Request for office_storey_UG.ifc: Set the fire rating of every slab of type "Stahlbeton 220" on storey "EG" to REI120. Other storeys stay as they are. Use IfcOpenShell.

First a look at what the model holds.

```python
import ifcopenshell
import ifcopenshell.util.element

model = ifcopenshell.open("office_storey_UG.ifc")
print(model.schema)
storey = next(s for s in model.by_type("IfcBuildingStorey") if s.Name == "EG")
slabs = [e for e in ifcopenshell.util.element.get_decomposition(storey) if e.is_a("IfcSlab")]
seen = {}
for e in slabs:
    element_type = ifcopenshell.util.element.get_type(e)
    key = (element_type.Name if element_type != e and element_type else None, ifcopenshell.util.element.get_pset(e, "Pset_SlabCommon", "FireRating"))
    seen[key] = seen.get(key, 0) + 1
for (name, value), count in sorted(seen.items(), key=str):
    print(count, "x", name, "|", value)
```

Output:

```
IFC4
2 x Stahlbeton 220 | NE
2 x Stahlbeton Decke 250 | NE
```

```python
import ifcopenshell
import ifcopenshell.api.pset
import ifcopenshell.util.element

model = ifcopenshell.open("office_storey_UG.ifc")

storey = next(s for s in model.by_type("IfcBuildingStorey") if s.Name == "EG")
slabs = [e for e in ifcopenshell.util.element.get_decomposition(storey) if e.is_a("IfcSlab")]

count = 0
for e in slabs:
    element_type = ifcopenshell.util.element.get_type(e)
    if element_type in (None, e) or element_type.Name != "Stahlbeton 220":
        continue
    # add_pset returns the element's existing set when there is one.
    pset = ifcopenshell.api.pset.add_pset(model, product=e, name="Pset_SlabCommon")
    ifcopenshell.api.pset.edit_pset(model, pset=pset, properties={"FireRating": "REI120"})
    count += 1

print(count, "slabs updated")

model.write("office_storey_UG_edited.ifc")
```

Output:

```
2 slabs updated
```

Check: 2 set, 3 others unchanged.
